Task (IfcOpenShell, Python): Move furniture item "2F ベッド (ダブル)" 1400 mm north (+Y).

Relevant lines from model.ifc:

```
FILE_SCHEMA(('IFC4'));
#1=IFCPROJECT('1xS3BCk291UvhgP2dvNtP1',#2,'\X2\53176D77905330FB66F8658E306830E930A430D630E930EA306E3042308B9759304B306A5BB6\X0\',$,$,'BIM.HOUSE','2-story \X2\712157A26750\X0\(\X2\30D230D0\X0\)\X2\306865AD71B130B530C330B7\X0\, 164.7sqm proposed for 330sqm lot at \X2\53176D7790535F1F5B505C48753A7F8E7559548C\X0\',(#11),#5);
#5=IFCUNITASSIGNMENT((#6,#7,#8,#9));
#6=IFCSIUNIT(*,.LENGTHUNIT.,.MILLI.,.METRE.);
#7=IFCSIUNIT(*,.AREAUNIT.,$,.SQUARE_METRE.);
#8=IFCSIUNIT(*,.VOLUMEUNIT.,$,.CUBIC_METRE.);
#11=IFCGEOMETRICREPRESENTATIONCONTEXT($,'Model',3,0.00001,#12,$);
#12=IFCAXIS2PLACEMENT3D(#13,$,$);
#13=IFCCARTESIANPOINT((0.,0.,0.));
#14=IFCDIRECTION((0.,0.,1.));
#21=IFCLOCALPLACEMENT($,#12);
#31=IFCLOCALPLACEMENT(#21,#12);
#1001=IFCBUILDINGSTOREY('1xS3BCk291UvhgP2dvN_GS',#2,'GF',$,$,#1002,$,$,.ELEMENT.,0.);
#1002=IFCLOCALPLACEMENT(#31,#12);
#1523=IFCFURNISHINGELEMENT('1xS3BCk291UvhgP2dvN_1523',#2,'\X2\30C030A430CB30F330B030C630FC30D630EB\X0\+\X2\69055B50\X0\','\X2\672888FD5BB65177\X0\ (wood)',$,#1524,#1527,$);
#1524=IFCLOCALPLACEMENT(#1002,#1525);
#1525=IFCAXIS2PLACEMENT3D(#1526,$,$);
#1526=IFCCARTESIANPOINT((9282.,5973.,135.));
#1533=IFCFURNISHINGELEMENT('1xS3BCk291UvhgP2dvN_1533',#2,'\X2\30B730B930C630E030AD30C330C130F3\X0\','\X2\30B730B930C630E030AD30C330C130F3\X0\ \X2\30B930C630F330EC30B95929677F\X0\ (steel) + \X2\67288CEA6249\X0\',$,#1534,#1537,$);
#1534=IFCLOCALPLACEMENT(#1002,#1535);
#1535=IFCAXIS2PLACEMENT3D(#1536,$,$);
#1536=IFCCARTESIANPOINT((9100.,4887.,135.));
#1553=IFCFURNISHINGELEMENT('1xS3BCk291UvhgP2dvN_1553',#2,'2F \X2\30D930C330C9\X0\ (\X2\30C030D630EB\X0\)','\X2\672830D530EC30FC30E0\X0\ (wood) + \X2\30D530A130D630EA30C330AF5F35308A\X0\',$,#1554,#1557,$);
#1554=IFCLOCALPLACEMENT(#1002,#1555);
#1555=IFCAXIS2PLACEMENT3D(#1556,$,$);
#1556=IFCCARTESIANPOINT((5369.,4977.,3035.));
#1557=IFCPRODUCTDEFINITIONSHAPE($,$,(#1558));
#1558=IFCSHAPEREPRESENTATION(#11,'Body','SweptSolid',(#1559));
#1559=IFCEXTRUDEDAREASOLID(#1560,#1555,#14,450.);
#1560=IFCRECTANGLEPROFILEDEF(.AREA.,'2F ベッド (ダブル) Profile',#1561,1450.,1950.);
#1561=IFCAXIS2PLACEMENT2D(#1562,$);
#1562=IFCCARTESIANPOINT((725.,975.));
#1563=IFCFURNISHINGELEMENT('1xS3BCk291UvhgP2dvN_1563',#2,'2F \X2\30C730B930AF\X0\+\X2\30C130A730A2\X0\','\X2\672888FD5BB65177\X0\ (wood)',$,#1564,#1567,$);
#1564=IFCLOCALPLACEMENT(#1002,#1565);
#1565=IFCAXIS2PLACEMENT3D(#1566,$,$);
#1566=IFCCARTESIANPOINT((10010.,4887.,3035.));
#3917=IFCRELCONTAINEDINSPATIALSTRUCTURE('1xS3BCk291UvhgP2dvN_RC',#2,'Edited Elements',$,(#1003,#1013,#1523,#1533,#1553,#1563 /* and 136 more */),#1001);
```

```python
import ifcopenshell
import ifcopenshell.api.geometry
import ifcopenshell.util.placement
import ifcopenshell.util.unit

model = ifcopenshell.open("model.ifc")
unit_scale = ifcopenshell.util.unit.calculate_unit_scale(model)

item = model.by_guid("1xS3BCk291UvhgP2dvN_1553")
matrix = ifcopenshell.util.placement.get_local_placement(item.ObjectPlacement)
matrix[1, 3] += 1.4 / unit_scale
ifcopenshell.api.geometry.edit_object_placement(model, product=item, matrix=matrix, is_si=False)

print(ifcopenshell.util.placement.get_local_placement(item.ObjectPlacement).round(3) + 0.0)

model.write("model_v2.ifc")
```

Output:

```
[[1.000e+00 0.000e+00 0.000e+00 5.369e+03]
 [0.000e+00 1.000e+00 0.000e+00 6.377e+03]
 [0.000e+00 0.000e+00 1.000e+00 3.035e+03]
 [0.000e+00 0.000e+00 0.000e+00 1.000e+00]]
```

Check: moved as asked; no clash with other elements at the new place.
